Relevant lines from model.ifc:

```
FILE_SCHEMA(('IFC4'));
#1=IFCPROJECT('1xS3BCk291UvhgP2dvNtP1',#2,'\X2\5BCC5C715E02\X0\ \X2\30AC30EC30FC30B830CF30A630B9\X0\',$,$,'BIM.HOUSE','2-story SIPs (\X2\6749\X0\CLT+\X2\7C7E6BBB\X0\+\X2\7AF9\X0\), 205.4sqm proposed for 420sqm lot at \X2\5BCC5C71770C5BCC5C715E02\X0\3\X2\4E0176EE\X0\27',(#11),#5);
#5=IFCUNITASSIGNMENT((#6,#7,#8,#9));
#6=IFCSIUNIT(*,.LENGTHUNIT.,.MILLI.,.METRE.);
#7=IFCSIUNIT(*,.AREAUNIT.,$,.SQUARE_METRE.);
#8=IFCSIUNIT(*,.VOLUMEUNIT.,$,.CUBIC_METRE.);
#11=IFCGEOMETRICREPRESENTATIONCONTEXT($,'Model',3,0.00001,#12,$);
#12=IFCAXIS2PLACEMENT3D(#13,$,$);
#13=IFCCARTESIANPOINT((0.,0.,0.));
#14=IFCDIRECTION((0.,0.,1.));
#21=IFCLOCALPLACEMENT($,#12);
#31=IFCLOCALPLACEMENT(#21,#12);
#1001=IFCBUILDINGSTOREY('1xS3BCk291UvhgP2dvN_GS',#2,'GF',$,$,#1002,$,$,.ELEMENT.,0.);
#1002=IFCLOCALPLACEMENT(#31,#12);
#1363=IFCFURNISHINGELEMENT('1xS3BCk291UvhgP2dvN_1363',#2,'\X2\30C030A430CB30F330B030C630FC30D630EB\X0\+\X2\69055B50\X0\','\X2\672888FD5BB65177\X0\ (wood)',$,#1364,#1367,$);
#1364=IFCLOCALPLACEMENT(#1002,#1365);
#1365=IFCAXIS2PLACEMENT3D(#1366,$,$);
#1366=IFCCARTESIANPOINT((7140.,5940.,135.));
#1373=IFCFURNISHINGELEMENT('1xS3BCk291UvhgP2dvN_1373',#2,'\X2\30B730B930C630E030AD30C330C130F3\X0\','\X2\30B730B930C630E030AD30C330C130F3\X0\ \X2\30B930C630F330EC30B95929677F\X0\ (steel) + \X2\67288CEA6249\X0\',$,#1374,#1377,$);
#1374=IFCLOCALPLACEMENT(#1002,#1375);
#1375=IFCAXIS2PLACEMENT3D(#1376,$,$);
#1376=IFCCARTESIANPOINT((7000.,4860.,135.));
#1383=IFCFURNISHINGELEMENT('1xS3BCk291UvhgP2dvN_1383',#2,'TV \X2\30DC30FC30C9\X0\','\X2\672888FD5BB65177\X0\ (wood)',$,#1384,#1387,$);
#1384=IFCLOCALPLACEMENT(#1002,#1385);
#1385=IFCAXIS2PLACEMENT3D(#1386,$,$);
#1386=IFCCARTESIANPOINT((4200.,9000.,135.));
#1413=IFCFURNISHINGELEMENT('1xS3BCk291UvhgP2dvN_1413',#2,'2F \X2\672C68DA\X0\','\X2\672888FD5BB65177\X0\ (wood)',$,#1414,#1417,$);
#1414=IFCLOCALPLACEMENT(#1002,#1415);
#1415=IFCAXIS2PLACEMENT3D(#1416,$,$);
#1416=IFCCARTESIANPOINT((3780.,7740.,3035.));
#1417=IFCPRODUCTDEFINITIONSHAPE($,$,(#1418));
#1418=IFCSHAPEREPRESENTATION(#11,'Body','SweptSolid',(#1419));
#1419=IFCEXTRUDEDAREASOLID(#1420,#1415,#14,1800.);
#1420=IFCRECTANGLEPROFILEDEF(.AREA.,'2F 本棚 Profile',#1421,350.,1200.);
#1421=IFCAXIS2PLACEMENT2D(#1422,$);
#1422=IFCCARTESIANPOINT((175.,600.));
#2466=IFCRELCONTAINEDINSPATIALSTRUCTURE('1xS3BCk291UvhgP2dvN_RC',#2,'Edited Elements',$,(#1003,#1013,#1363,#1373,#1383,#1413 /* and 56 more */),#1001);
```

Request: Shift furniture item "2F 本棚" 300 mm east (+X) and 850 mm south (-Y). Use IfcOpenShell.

```python
import ifcopenshell
import ifcopenshell.api.geometry
import ifcopenshell.util.placement

model = ifcopenshell.open("model.ifc")

item = model.by_id(1413)
matrix = ifcopenshell.util.placement.get_local_placement(item.ObjectPlacement)
matrix[0, 3] += 300.0
matrix[1, 3] -= 850.0
ifcopenshell.api.geometry.edit_object_placement(model, product=item, matrix=matrix, is_si=False)

print(ifcopenshell.util.placement.get_local_placement(item.ObjectPlacement).round(3) + 0.0)

model.write("model_updated.ifc")
```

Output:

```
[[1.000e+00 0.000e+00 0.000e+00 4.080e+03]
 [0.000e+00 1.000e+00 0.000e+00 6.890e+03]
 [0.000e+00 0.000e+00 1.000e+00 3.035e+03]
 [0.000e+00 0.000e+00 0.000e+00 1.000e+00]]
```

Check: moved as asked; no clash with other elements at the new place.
